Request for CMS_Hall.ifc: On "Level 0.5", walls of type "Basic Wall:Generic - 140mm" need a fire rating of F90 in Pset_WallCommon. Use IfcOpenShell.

First a look at what the model holds.

```python
import ifcopenshell
import ifcopenshell.util.element

model = ifcopenshell.open("CMS_Hall.ifc")
print(model.schema)
storey = next(s for s in model.by_type("IfcBuildingStorey") if s.Name == "Level 0.5")
walls = [e for e in ifcopenshell.util.element.get_decomposition(storey) if e.is_a("IfcWall")]
seen = {}
for e in walls:
    element_type = ifcopenshell.util.element.get_type(e)
    key = (element_type.Name if element_type != e and element_type else None, ifcopenshell.util.element.get_pset(e, "Pset_WallCommon", "FireRating"))
    seen[key] = seen.get(key, 0) + 1
for (name, value), count in sorted(seen.items(), key=str):
    print(count, "x", name, "|", value)
```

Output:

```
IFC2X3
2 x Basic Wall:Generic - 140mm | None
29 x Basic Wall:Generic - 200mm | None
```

```python
import ifcopenshell
import ifcopenshell.api.pset
import ifcopenshell.util.element

model = ifcopenshell.open("CMS_Hall.ifc")

storey = next(s for s in model.by_type("IfcBuildingStorey") if s.Name == "Level 0.5")
walls = [e for e in ifcopenshell.util.element.get_decomposition(storey) if e.is_a("IfcWall")]

count = 0
for e in walls:
    element_type = ifcopenshell.util.element.get_type(e)
    if element_type in (None, e) or element_type.Name != "Basic Wall:Generic - 140mm":
        continue
    # add_pset returns the element's existing set when there is one.
    pset = ifcopenshell.api.pset.add_pset(model, product=e, name="Pset_WallCommon")
    ifcopenshell.api.pset.edit_pset(model, pset=pset, properties={"FireRating": "F90"})
    count += 1

print(count, "walls updated")

model.write("CMS_Hall_updated.ifc")
```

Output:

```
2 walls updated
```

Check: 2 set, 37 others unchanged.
